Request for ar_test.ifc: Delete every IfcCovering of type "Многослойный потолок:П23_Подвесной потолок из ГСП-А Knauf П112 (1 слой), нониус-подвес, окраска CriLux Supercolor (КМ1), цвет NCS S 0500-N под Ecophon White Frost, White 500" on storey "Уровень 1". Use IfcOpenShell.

First a look at what the model holds.

```python
import ifcopenshell
import ifcopenshell.util.element

model = ifcopenshell.open("ar_test.ifc")
print(model.schema)
storey = next(s for s in model.by_type("IfcBuildingStorey") if s.Name == "Уровень 1")
coverings = [e for e in ifcopenshell.util.element.get_decomposition(storey) if e.is_a("IfcCovering")]
seen = {}
for e in coverings:
    element_type = ifcopenshell.util.element.get_type(e)
    name = element_type.Name if element_type not in (None, e) else None
    seen[name] = seen.get(name, 0) + 1
for name, count in sorted(seen.items(), key=str):
    print(count, "x", name)
```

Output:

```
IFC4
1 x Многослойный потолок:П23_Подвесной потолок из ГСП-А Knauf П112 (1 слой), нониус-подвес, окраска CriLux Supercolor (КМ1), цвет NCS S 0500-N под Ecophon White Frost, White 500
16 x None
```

```python
import ifcopenshell
import ifcopenshell.api.root
import ifcopenshell.util.element

model = ifcopenshell.open("ar_test.ifc")

storey = next(s for s in model.by_type("IfcBuildingStorey") if s.Name == "Уровень 1")
coverings = [e for e in ifcopenshell.util.element.get_decomposition(storey) if e.is_a("IfcCovering")]
targets = [e for e in coverings if (t := ifcopenshell.util.element.get_type(e)) not in (None, e) and t.Name == "Многослойный потолок:П23_Подвесной потолок из ГСП-А Knauf П112 (1 слой), нониус-подвес, окраска CriLux Supercolor (КМ1), цвет NCS S 0500-N под Ecophon White Frost, White 500"]

for e in targets:
    ifcopenshell.api.root.remove_product(model, product=e)
print(len(targets), "removed")

model.write("ar_test-out.ifc")
```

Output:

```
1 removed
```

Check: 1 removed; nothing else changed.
